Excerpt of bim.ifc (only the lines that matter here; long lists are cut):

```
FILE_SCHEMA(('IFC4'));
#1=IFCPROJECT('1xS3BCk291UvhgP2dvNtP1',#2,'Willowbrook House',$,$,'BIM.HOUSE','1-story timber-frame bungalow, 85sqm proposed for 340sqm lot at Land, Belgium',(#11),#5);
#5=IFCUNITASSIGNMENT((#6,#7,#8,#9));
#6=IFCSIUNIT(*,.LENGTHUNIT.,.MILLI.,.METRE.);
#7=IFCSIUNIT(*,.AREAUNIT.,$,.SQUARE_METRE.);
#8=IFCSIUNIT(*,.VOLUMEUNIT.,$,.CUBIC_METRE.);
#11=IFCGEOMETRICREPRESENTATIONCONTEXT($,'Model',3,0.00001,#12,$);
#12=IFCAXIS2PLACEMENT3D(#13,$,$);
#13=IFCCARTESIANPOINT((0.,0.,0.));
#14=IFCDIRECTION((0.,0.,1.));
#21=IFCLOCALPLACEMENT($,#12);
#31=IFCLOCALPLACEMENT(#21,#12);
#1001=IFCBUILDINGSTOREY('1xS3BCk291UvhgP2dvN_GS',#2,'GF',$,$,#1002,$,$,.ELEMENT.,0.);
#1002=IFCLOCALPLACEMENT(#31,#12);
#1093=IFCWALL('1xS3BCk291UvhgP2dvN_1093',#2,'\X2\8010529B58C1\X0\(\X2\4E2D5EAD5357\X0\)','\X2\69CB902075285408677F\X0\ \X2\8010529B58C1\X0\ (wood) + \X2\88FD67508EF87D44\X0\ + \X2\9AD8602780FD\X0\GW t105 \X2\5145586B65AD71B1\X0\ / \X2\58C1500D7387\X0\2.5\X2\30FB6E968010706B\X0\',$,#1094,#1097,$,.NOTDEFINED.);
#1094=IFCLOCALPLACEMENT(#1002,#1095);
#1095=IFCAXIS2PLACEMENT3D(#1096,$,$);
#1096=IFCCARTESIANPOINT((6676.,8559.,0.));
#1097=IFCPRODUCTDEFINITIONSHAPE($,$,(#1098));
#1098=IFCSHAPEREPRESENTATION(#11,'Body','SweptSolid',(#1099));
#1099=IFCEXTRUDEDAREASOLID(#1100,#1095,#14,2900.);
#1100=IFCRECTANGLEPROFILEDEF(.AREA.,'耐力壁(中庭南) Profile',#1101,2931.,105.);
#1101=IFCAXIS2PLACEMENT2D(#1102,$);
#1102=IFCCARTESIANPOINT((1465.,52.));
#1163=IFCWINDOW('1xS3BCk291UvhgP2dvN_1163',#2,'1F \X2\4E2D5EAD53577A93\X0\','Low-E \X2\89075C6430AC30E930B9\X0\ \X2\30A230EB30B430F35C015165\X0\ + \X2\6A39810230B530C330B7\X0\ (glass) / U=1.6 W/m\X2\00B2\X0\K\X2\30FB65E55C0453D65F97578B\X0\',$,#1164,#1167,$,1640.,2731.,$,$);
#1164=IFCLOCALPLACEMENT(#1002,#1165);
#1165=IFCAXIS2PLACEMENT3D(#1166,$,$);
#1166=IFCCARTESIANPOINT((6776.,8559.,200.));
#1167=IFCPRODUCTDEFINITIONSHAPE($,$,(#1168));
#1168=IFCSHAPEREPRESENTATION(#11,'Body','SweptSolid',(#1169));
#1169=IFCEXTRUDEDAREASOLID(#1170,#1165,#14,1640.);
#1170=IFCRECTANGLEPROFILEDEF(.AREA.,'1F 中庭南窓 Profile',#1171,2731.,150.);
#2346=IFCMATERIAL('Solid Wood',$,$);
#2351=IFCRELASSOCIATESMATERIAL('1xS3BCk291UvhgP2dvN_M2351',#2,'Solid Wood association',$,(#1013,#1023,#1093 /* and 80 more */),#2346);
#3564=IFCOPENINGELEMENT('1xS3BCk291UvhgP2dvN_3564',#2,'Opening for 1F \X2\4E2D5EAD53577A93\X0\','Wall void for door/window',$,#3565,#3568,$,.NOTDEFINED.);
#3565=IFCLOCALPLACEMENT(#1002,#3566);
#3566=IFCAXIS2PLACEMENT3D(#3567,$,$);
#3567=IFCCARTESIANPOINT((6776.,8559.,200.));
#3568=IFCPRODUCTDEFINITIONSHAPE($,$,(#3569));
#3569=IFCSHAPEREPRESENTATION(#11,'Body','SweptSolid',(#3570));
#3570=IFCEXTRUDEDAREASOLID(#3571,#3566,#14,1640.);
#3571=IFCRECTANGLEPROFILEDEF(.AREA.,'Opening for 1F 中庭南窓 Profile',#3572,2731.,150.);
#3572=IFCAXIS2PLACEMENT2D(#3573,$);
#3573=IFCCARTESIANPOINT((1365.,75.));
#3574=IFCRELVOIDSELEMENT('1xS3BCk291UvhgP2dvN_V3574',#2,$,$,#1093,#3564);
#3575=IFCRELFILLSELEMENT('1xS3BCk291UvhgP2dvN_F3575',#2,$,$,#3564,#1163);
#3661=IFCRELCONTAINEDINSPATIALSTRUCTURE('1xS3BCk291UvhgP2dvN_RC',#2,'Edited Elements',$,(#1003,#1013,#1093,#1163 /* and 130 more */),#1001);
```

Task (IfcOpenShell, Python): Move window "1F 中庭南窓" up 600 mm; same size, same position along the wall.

```python
import numpy as np
import ifcopenshell
import ifcopenshell.api.geometry
import ifcopenshell.util.placement
import ifcopenshell.util.unit

model = ifcopenshell.open("bim.ifc")
unit_scale = ifcopenshell.util.unit.calculate_unit_scale(model)

window = model.by_guid("1xS3BCk291UvhgP2dvN_1163")
opening = window.FillsVoids[0].RelatingOpeningElement
dz = 0.6 / unit_scale

shift = np.array([0.0, 0.0, dz])
# The window is not placed relative to its opening, so move both.
for product in (opening, window):
    matrix = ifcopenshell.util.placement.get_local_placement(product.ObjectPlacement)
    matrix[:3, 3] += shift
    ifcopenshell.api.geometry.edit_object_placement(model, product=product, matrix=matrix, is_si=False)

print(f"moved by {dz * unit_scale:+.3f} m")

model.write("bim-out.ifc")
```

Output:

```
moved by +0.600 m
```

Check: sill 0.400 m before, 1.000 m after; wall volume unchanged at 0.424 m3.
